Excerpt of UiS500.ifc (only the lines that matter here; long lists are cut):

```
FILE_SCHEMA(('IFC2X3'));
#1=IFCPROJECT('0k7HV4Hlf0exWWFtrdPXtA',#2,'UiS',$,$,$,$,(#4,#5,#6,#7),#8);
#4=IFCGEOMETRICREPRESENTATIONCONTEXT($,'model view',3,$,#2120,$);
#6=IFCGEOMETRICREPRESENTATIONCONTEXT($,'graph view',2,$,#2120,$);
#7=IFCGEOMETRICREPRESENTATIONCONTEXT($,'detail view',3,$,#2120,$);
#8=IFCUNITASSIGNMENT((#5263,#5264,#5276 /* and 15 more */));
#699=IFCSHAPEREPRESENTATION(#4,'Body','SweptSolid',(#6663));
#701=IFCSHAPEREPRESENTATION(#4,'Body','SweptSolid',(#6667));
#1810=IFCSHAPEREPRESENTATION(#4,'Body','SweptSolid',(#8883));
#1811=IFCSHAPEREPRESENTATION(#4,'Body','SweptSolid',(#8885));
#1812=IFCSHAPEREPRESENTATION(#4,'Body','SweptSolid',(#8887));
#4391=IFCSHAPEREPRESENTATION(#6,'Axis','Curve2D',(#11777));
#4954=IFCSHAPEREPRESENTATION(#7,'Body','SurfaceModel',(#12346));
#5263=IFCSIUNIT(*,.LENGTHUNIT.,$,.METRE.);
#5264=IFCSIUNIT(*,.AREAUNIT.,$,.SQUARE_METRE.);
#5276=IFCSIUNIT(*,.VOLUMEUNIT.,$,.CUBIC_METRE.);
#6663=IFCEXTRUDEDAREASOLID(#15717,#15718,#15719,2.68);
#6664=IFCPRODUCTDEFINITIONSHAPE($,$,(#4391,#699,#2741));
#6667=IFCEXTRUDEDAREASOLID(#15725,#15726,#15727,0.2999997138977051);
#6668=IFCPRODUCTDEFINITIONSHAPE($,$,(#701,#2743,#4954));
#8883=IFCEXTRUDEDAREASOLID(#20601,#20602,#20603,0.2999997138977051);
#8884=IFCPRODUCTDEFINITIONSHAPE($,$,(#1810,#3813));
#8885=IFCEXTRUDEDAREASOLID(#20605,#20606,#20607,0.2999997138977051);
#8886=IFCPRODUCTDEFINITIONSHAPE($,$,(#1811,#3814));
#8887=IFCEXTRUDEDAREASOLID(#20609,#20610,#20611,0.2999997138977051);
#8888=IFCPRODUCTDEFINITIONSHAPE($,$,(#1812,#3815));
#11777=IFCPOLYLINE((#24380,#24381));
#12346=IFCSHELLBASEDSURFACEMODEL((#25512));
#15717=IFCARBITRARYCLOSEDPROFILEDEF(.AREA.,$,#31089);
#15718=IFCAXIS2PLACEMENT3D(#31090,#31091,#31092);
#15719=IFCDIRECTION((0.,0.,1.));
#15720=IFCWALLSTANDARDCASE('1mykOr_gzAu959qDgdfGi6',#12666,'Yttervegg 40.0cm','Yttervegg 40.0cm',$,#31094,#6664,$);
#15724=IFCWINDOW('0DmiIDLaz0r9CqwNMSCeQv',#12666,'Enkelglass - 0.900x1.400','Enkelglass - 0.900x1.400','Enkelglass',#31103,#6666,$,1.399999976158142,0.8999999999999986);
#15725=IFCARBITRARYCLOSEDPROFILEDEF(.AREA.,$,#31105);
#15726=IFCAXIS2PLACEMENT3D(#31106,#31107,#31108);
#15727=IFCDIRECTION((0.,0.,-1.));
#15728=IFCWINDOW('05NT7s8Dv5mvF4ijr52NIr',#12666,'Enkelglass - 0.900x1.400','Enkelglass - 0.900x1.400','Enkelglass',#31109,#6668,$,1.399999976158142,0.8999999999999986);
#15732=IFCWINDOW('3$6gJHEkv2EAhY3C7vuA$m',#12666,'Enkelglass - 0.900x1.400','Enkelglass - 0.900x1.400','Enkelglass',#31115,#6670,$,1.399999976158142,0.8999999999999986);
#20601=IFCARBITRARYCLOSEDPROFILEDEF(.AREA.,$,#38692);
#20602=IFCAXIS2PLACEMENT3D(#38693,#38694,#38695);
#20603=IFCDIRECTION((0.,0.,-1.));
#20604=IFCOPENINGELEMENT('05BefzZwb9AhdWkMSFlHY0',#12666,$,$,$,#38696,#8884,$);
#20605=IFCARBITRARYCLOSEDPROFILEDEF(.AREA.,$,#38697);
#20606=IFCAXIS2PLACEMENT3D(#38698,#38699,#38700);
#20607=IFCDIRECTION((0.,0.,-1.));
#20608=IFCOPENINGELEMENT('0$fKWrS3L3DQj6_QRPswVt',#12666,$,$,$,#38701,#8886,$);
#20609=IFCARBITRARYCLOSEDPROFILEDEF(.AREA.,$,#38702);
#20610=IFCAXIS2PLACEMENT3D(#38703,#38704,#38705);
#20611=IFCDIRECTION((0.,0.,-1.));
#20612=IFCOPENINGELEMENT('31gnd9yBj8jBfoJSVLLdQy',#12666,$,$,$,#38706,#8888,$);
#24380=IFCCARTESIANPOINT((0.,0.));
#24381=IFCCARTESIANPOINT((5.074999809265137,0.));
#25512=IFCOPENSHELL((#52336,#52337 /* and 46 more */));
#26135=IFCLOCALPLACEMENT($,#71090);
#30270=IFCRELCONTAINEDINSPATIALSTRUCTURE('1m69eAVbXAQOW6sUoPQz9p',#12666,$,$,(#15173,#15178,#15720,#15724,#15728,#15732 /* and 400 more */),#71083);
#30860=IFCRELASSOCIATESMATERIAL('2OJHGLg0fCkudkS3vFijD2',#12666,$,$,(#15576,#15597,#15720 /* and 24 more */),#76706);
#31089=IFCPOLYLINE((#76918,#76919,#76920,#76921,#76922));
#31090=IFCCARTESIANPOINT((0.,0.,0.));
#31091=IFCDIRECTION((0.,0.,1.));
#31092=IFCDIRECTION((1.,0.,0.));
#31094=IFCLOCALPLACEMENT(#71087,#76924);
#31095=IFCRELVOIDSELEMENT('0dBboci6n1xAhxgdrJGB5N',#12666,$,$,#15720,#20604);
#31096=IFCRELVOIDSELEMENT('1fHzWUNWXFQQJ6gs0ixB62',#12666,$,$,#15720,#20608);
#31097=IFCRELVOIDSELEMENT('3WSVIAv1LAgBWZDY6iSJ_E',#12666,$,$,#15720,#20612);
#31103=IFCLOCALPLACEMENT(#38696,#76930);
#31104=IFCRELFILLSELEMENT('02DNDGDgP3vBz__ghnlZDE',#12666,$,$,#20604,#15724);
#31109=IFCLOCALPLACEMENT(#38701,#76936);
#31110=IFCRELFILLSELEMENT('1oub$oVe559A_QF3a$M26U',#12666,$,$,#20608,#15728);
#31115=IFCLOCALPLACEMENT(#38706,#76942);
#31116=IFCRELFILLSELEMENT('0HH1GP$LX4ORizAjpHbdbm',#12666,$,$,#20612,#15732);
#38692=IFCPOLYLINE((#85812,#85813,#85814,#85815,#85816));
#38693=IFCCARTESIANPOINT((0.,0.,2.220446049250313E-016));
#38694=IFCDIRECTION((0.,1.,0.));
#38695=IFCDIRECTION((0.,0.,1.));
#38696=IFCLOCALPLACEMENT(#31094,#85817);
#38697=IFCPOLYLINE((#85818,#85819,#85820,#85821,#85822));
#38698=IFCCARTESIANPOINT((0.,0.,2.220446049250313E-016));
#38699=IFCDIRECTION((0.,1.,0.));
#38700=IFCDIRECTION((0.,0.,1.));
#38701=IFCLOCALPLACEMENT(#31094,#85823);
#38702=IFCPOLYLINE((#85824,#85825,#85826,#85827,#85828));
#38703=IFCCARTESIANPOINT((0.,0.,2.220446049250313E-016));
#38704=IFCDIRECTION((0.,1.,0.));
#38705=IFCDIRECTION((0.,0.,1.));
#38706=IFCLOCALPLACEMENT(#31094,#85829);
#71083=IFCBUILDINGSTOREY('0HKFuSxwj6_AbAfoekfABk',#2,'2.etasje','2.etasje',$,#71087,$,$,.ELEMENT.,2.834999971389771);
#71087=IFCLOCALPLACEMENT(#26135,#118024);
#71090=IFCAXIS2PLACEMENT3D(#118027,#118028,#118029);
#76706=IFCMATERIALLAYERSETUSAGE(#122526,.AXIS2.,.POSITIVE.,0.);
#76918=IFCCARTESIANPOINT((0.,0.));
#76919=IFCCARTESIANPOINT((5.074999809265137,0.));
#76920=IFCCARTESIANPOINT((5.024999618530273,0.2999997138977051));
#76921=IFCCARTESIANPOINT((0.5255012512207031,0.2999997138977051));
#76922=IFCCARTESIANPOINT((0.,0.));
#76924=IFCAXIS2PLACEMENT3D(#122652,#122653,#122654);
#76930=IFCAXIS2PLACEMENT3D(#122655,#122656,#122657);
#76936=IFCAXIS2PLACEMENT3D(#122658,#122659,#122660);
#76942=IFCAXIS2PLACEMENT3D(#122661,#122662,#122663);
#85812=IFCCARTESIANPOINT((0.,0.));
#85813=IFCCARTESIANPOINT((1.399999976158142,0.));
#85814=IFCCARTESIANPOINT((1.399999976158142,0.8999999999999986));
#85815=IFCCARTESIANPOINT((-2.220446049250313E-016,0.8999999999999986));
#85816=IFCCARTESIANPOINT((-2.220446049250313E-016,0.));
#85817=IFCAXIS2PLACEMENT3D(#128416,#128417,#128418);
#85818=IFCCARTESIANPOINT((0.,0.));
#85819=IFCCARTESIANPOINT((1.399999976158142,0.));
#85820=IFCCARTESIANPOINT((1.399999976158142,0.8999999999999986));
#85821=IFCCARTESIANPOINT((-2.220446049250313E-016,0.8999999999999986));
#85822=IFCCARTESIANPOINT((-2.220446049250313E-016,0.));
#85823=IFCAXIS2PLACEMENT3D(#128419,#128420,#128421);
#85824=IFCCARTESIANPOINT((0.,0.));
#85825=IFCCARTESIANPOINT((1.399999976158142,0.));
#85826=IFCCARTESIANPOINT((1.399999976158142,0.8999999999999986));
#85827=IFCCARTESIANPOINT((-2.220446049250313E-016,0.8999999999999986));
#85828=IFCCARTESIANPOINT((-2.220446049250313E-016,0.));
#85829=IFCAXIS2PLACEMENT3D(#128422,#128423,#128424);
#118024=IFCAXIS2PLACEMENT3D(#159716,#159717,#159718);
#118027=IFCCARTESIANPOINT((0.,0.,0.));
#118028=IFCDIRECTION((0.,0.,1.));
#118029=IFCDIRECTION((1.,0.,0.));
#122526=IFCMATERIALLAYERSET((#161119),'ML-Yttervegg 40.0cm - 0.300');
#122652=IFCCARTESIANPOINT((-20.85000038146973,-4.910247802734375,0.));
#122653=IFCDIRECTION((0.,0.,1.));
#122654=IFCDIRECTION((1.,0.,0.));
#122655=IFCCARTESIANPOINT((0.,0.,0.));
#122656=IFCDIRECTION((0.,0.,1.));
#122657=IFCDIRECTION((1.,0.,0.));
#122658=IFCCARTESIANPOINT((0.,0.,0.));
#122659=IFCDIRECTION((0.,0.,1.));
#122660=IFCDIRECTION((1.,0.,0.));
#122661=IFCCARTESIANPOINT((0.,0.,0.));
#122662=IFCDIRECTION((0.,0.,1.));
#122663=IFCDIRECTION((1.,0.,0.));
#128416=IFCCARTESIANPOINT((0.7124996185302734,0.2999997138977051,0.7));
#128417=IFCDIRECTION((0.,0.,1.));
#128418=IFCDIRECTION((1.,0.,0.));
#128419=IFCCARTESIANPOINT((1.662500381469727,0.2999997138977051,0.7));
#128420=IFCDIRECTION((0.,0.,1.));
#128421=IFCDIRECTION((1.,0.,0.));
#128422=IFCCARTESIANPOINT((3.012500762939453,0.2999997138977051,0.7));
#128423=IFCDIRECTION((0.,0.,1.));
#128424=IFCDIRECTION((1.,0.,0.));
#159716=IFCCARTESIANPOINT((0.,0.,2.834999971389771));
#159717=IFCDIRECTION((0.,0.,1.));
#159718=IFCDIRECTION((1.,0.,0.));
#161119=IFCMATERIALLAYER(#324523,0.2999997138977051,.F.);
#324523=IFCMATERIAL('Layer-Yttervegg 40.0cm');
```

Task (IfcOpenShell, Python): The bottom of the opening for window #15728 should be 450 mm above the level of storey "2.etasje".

```python
import numpy as np
import ifcopenshell
import ifcopenshell.api.geometry
import ifcopenshell.geom
import ifcopenshell.util.element
import ifcopenshell.util.placement
import ifcopenshell.util.shape
import ifcopenshell.util.unit

model = ifcopenshell.open("UiS500.ifc")
unit_scale = ifcopenshell.util.unit.calculate_unit_scale(model)

window = model.by_guid("05NT7s8Dv5mvF4ijr52NIr")
opening = window.FillsVoids[0].RelatingOpeningElement
storey = ifcopenshell.util.element.get_container(window, ifc_class="IfcBuildingStorey")
level = ifcopenshell.util.placement.get_local_placement(storey.ObjectPlacement)[2, 3]

# The opening's origin need not be at the sill, so measure its lowest point.
shape = ifcopenshell.geom.create_shape(ifcopenshell.geom.settings(), opening)
bottom = ifcopenshell.util.shape.get_shape_bottom_elevation(shape, shape.geometry) / unit_scale
dz = level + 0.45 - bottom

shift = np.array([0.0, 0.0, dz])
# The window is placed relative to its opening, so it follows when the opening moves.
matrix = ifcopenshell.util.placement.get_local_placement(opening.ObjectPlacement)
matrix[:3, 3] += shift
ifcopenshell.api.geometry.edit_object_placement(
    model, product=opening, matrix=matrix, is_si=False, should_transform_children=True
)

print(f"moved by {dz * unit_scale:+.3f} m")

model.write("UiS500_updated.ifc")
```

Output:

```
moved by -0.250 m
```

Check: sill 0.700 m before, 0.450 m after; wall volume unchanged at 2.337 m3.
